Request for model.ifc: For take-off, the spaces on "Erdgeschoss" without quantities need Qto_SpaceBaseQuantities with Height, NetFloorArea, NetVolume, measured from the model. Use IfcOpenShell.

First a look at what the model holds.

```python
import ifcopenshell
import ifcopenshell.util.element
import ifcopenshell.util.unit

model = ifcopenshell.open("model.ifc")
print(model.schema)
for unit_type in ("LENGTHUNIT", "AREAUNIT", "VOLUMEUNIT"):
    print(unit_type, ifcopenshell.util.unit.calculate_unit_scale(model, unit_type))
storey = next(s for s in model.by_type("IfcBuildingStorey") if s.Name == "Erdgeschoss")
spaces = [e for e in ifcopenshell.util.element.get_decomposition(storey) if e.is_a("IfcSpace")]
for e in sorted(spaces, key=lambda e: e.id()):
    print(e.id(), e.is_a(), e.Name, list(ifcopenshell.util.element.get_psets(e, qtos_only=True)), sep=" | ")
```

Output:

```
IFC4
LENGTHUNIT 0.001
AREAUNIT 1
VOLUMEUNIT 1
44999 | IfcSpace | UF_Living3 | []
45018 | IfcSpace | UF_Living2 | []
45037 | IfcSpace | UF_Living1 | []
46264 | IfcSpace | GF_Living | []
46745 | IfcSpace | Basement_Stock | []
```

```python
import ifcopenshell
import ifcopenshell.api.pset
import ifcopenshell.geom
import ifcopenshell.util.element
import ifcopenshell.util.shape
import ifcopenshell.util.unit

model = ifcopenshell.open("model.ifc")
unit_scale = ifcopenshell.util.unit.calculate_unit_scale(model)
area_scale = ifcopenshell.util.unit.calculate_unit_scale(model, "AREAUNIT")
volume_scale = ifcopenshell.util.unit.calculate_unit_scale(model, "VOLUMEUNIT")
settings = ifcopenshell.geom.settings()

storey = next(s for s in model.by_type("IfcBuildingStorey") if s.Name == "Erdgeschoss")
spaces = [e for e in ifcopenshell.util.element.get_decomposition(storey) if e.is_a("IfcSpace")]

for e in sorted(spaces, key=lambda e: e.id()):
    if ifcopenshell.util.element.get_psets(e, qtos_only=True, should_inherit=False):
        continue
    # Geometry comes back in metres, in the element's own axes.
    shape = ifcopenshell.geom.create_shape(settings, e)
    values = {
        "Height": ifcopenshell.util.shape.get_z(shape.geometry) / unit_scale,
        "NetFloorArea": ifcopenshell.util.shape.get_footprint_area(shape.geometry) / area_scale,
        "NetVolume": ifcopenshell.util.shape.get_volume(shape.geometry) / volume_scale,
    }
    qto = ifcopenshell.api.pset.add_qto(model, product=e, name="Qto_SpaceBaseQuantities")
    ifcopenshell.api.pset.edit_qto(model, qto=qto, properties=values)
    print(e.id(), {k: round(v, 3) for k, v in values.items()})

model.write("model-out.ifc")
```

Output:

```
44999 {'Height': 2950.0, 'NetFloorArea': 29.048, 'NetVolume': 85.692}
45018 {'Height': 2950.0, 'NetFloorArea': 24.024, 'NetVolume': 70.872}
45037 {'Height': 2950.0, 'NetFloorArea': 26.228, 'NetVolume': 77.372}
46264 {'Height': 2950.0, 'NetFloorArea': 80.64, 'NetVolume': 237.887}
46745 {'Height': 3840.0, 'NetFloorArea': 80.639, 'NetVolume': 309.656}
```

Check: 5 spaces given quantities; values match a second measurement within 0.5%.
